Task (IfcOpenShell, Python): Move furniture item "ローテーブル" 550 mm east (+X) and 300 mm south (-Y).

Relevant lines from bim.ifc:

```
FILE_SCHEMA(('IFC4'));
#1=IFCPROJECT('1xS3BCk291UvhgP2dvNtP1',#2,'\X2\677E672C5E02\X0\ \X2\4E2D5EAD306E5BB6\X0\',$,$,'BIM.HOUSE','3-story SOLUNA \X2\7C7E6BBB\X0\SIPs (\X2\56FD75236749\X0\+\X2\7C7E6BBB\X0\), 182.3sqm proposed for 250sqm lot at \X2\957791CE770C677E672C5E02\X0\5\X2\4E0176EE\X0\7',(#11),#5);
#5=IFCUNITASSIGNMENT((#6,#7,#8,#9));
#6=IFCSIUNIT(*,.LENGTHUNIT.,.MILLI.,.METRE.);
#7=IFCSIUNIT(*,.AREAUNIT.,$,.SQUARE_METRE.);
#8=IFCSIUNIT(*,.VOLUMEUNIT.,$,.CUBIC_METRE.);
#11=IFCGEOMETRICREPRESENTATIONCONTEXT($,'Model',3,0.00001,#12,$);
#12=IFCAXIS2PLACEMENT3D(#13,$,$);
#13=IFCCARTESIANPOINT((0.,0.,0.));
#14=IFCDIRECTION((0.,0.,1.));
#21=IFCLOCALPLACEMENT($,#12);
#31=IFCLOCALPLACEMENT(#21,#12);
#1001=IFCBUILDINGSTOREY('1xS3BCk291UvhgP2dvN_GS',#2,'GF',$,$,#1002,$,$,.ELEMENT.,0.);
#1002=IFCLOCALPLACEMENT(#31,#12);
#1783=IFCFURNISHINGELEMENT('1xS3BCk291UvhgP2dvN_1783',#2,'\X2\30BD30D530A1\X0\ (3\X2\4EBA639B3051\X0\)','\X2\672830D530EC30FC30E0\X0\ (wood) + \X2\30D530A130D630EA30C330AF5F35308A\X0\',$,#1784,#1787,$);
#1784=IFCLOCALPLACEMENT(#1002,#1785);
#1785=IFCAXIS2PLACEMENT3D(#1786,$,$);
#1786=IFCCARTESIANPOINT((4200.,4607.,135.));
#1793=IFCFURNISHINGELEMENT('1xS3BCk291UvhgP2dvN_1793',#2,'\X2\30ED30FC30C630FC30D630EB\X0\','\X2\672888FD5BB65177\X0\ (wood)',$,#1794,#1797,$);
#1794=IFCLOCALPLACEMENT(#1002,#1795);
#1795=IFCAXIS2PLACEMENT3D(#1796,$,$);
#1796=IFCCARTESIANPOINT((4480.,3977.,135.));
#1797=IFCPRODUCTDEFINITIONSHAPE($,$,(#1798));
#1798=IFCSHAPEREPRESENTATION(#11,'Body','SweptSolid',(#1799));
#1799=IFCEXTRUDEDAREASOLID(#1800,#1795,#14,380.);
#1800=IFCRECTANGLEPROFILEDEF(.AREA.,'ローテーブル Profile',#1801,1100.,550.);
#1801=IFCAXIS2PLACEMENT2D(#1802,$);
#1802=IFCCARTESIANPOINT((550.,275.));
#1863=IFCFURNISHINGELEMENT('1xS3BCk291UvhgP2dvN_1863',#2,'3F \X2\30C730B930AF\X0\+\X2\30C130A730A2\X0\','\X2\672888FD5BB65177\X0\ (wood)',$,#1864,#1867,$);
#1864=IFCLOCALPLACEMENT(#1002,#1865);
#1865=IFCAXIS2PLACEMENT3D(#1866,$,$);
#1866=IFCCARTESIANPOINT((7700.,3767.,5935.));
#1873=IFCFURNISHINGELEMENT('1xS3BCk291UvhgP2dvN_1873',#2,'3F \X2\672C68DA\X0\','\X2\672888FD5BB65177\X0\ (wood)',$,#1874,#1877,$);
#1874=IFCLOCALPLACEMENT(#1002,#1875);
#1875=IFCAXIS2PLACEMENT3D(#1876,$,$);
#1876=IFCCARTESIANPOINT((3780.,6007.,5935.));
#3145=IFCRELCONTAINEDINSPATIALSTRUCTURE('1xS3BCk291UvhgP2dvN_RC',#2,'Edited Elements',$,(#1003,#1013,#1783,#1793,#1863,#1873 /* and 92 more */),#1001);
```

```python
import ifcopenshell
import ifcopenshell.api.geometry
import ifcopenshell.util.placement
import ifcopenshell.util.unit

model = ifcopenshell.open("bim.ifc")
unit_scale = ifcopenshell.util.unit.calculate_unit_scale(model)

item = model.by_id(1793)
matrix = ifcopenshell.util.placement.get_local_placement(item.ObjectPlacement)
matrix[0, 3] += 0.55 / unit_scale
matrix[1, 3] -= 0.3 / unit_scale
ifcopenshell.api.geometry.edit_object_placement(model, product=item, matrix=matrix, is_si=False)

print(ifcopenshell.util.placement.get_local_placement(item.ObjectPlacement).round(3) + 0.0)

model.write("bim_updated.ifc")
```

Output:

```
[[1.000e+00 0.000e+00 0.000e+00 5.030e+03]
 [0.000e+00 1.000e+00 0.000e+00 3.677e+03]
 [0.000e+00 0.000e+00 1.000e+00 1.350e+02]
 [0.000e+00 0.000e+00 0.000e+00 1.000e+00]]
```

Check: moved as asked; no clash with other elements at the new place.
